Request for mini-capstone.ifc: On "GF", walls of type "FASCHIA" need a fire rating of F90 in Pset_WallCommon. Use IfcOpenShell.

First a look at what the model holds.

```python
import ifcopenshell
import ifcopenshell.util.element

model = ifcopenshell.open("mini-capstone.ifc")
print(model.schema)
storey = next(s for s in model.by_type("IfcBuildingStorey") if s.Name == "GF")
walls = [e for e in ifcopenshell.util.element.get_decomposition(storey) if e.is_a("IfcWall")]
seen = {}
for e in walls:
    element_type = ifcopenshell.util.element.get_type(e)
    key = (element_type.Name if element_type != e and element_type else None, ifcopenshell.util.element.get_pset(e, "Pset_WallCommon", "FireRating"))
    seen[key] = seen.get(key, 0) + 1
for (name, value), count in sorted(seen.items(), key=str):
    print(count, "x", name, "|", value)
```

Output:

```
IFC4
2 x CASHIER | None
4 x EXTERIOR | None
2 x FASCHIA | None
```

```python
import ifcopenshell
import ifcopenshell.api.pset
import ifcopenshell.util.element

model = ifcopenshell.open("mini-capstone.ifc")

storey = next(s for s in model.by_type("IfcBuildingStorey") if s.Name == "GF")
walls = [e for e in ifcopenshell.util.element.get_decomposition(storey) if e.is_a("IfcWall")]

count = 0
for e in walls:
    element_type = ifcopenshell.util.element.get_type(e)
    if element_type in (None, e) or element_type.Name != "FASCHIA":
        continue
    # add_pset returns the element's existing set when there is one.
    pset = ifcopenshell.api.pset.add_pset(model, product=e, name="Pset_WallCommon")
    ifcopenshell.api.pset.edit_pset(model, pset=pset, properties={"FireRating": "F90"})
    count += 1

print(count, "walls updated")

model.write("mini-capstone-out.ifc")
```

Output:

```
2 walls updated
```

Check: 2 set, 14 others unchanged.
